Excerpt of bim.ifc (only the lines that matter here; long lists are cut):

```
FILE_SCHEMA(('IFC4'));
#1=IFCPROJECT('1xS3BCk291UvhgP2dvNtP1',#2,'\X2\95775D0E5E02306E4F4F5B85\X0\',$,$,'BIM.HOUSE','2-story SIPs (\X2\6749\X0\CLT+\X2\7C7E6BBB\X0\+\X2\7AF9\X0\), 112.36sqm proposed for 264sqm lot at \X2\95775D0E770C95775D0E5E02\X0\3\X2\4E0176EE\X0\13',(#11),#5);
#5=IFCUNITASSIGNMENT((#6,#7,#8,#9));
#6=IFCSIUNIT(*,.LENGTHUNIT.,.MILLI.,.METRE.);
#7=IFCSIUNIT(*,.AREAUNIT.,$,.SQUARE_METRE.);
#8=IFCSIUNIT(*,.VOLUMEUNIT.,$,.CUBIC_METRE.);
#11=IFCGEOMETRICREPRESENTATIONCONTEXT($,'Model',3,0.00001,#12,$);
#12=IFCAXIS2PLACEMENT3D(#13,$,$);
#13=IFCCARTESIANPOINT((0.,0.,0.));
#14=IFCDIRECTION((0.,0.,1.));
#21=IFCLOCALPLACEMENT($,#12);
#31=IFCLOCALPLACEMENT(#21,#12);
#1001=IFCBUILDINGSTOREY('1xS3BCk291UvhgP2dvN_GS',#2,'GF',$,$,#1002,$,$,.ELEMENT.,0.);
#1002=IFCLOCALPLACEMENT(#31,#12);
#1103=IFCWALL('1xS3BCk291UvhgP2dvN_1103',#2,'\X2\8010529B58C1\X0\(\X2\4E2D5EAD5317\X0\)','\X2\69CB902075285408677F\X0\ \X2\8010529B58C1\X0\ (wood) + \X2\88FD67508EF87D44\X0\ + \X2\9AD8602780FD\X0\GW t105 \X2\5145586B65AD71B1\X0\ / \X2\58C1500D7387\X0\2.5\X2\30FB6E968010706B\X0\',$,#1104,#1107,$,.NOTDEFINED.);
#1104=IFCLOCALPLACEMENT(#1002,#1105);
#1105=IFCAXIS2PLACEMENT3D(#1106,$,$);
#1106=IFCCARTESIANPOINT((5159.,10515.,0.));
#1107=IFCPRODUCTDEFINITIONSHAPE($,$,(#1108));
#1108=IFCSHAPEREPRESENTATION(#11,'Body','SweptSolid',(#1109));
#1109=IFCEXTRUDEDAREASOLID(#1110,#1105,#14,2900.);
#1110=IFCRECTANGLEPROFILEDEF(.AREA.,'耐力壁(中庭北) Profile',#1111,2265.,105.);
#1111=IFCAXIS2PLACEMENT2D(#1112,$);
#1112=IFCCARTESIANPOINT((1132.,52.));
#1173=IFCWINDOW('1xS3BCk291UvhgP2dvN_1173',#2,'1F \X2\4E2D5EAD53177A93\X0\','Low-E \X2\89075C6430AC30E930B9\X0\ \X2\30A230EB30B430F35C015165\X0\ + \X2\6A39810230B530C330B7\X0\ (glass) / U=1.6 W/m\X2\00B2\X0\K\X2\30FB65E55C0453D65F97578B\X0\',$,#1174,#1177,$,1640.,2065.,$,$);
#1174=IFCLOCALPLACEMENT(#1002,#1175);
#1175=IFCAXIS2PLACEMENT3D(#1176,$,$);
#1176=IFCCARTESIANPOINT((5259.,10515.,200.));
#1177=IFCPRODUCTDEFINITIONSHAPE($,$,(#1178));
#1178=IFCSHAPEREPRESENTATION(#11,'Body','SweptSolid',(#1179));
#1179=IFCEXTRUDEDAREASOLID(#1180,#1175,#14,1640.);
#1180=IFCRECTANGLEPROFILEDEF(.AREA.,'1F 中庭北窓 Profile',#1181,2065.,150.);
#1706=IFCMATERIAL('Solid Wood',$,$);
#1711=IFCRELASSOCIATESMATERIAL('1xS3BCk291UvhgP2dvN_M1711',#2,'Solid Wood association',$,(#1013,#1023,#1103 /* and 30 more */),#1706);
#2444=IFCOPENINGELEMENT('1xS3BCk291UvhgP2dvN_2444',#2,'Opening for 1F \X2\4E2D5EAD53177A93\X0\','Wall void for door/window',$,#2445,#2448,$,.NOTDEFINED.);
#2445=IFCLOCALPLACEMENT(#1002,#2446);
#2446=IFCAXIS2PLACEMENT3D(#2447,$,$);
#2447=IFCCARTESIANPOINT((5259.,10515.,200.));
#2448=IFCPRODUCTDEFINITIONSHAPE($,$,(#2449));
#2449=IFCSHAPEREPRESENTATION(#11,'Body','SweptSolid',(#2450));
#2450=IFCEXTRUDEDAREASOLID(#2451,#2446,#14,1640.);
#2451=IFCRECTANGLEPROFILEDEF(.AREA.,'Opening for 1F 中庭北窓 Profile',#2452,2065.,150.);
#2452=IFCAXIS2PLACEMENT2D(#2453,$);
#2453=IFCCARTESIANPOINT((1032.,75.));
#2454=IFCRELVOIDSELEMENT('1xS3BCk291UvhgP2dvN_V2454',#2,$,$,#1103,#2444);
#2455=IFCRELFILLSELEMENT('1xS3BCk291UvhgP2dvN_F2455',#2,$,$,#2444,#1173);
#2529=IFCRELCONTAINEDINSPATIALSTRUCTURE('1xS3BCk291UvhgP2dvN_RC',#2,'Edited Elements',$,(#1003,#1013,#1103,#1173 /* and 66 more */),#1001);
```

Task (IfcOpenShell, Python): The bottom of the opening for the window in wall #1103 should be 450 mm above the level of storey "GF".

```python
import numpy as np
import ifcopenshell
import ifcopenshell.api.geometry
import ifcopenshell.geom
import ifcopenshell.util.element
import ifcopenshell.util.placement
import ifcopenshell.util.shape
import ifcopenshell.util.unit

model = ifcopenshell.open("bim.ifc")
unit_scale = ifcopenshell.util.unit.calculate_unit_scale(model)

window = model.by_guid("1xS3BCk291UvhgP2dvN_1173")
opening = window.FillsVoids[0].RelatingOpeningElement
storey = ifcopenshell.util.element.get_container(window, ifc_class="IfcBuildingStorey")
level = ifcopenshell.util.placement.get_local_placement(storey.ObjectPlacement)[2, 3]

# The opening's origin need not be at the sill, so measure its lowest point.
shape = ifcopenshell.geom.create_shape(ifcopenshell.geom.settings(), opening)
bottom = ifcopenshell.util.shape.get_shape_bottom_elevation(shape, shape.geometry) / unit_scale
dz = level + 0.45 / unit_scale - bottom

shift = np.array([0.0, 0.0, dz])
# The window is not placed relative to its opening, so move both.
for product in (opening, window):
    matrix = ifcopenshell.util.placement.get_local_placement(product.ObjectPlacement)
    matrix[:3, 3] += shift
    ifcopenshell.api.geometry.edit_object_placement(model, product=product, matrix=matrix, is_si=False)

print(f"moved by {dz * unit_scale:+.3f} m")

model.write("bim_v2.ifc")
```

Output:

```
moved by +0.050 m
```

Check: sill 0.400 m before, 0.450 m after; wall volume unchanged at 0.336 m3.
